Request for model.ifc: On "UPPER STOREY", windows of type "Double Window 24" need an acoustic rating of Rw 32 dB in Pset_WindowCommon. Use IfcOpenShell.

First a look at what the model holds.

```python
import ifcopenshell
import ifcopenshell.util.element

model = ifcopenshell.open("model.ifc")
print(model.schema)
storey = next(s for s in model.by_type("IfcBuildingStorey") if s.Name == "UPPER STOREY")
windows = [e for e in ifcopenshell.util.element.get_decomposition(storey) if e.is_a("IfcWindow")]
seen = {}
for e in windows:
    element_type = ifcopenshell.util.element.get_type(e)
    key = (element_type.Name if element_type != e and element_type else None, ifcopenshell.util.element.get_pset(e, "Pset_WindowCommon", "AcousticRating"))
    seen[key] = seen.get(key, 0) + 1
for (name, value), count in sorted(seen.items(), key=str):
    print(count, "x", name, "|", value)
```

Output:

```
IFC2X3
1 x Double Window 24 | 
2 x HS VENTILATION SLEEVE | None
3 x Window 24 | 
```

```python
import ifcopenshell
import ifcopenshell.api.pset
import ifcopenshell.util.element

model = ifcopenshell.open("model.ifc")

storey = next(s for s in model.by_type("IfcBuildingStorey") if s.Name == "UPPER STOREY")
windows = [e for e in ifcopenshell.util.element.get_decomposition(storey) if e.is_a("IfcWindow")]

count = 0
for e in windows:
    element_type = ifcopenshell.util.element.get_type(e)
    if element_type in (None, e) or element_type.Name != "Double Window 24":
        continue
    # add_pset returns the element's existing set when there is one.
    pset = ifcopenshell.api.pset.add_pset(model, product=e, name="Pset_WindowCommon")
    ifcopenshell.api.pset.edit_pset(model, pset=pset, properties={"AcousticRating": "Rw 32 dB"})
    count += 1

print(count, "windows updated")

model.write("model_v2.ifc")
```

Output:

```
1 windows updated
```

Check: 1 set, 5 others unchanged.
